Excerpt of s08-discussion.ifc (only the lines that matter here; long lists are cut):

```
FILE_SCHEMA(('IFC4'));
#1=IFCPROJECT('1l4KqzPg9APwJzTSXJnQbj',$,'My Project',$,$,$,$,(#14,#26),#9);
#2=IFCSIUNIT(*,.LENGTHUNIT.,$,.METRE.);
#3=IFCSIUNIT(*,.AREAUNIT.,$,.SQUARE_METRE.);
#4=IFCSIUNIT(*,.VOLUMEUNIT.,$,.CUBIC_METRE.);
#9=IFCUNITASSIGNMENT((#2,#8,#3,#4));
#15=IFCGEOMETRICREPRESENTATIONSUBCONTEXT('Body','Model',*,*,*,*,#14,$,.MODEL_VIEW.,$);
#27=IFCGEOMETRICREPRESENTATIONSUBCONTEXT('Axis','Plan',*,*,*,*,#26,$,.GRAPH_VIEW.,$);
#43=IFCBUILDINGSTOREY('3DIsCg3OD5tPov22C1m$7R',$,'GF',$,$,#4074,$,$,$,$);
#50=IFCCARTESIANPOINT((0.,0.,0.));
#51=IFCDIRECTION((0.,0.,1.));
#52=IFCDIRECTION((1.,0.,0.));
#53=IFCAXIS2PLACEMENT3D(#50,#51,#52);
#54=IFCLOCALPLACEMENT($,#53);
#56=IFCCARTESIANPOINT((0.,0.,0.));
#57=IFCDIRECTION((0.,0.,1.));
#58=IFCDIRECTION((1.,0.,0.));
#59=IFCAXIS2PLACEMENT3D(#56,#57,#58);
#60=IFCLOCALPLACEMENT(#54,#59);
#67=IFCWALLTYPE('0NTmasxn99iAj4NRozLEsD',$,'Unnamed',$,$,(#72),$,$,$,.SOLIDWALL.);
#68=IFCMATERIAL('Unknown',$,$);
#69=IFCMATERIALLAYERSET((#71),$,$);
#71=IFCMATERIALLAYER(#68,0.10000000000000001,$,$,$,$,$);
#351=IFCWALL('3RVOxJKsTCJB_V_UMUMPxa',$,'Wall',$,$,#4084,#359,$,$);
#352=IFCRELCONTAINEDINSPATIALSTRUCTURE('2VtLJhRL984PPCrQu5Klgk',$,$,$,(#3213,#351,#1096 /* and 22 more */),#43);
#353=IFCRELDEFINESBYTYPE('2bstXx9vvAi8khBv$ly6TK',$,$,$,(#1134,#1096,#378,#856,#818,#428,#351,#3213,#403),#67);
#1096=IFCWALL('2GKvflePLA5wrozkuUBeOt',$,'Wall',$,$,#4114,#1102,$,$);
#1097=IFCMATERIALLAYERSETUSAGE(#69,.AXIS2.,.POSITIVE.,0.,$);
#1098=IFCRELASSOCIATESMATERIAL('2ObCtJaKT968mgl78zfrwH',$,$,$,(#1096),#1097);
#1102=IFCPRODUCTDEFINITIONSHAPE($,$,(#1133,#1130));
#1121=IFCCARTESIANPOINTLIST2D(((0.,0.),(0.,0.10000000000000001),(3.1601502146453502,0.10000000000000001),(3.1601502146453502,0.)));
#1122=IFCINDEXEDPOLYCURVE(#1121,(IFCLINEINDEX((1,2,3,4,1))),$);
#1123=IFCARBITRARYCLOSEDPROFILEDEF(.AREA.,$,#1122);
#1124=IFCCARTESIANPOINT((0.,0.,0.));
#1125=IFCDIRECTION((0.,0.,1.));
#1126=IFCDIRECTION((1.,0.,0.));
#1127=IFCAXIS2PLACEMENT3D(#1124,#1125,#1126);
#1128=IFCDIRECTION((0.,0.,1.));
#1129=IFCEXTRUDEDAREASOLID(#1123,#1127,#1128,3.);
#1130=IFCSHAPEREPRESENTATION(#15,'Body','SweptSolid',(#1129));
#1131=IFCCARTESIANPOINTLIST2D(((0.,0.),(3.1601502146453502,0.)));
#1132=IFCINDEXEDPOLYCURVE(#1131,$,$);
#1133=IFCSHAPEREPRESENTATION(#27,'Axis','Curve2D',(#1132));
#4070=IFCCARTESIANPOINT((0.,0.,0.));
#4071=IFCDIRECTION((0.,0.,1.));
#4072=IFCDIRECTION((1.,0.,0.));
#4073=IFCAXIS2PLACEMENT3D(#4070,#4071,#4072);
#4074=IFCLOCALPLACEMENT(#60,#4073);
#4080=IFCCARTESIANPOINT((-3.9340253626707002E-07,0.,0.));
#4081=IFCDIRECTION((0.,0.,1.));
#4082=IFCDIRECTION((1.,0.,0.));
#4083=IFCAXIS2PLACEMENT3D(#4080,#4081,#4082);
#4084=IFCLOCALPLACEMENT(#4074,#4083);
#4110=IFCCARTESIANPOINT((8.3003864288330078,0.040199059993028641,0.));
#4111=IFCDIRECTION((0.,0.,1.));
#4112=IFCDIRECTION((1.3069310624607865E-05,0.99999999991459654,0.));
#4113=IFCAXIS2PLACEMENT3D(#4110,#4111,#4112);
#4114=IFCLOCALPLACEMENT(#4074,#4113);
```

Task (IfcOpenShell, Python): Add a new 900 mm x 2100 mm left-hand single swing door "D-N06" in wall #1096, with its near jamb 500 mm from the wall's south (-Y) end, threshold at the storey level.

```python
import numpy as np
import ifcopenshell
import ifcopenshell.api.feature
import ifcopenshell.api.geometry
import ifcopenshell.api.root
import ifcopenshell.api.spatial
import ifcopenshell.geom
import ifcopenshell.util.element
import ifcopenshell.util.placement
import ifcopenshell.util.representation
import ifcopenshell.util.shape
import ifcopenshell.util.unit

model = ifcopenshell.open("s08-discussion.ifc")
unit_scale = ifcopenshell.util.unit.calculate_unit_scale(model)
settings = ifcopenshell.geom.settings()


def volume(element):
    """Net volume in cubic metres, openings subtracted."""
    shape = ifcopenshell.geom.create_shape(settings, element)
    return ifcopenshell.util.shape.get_volume(shape.geometry)


wall = model.by_guid("2GKvflePLA5wrozkuUBeOt")
storey = ifcopenshell.util.element.get_container(wall, ifc_class="IfcBuildingStorey")
context = ifcopenshell.util.representation.get_context(model, "Model", "Body", "MODEL_VIEW")
before = volume(wall)

width, height, from_end, sill = 0.9, 2.1, 0.5, 0.0  # metres

# The wall runs along its own X axis, and the end named is its -X end.
wall_shape = ifcopenshell.geom.create_shape(settings, wall)
x, y, z = ifcopenshell.util.shape.get_vertices(wall_shape.geometry).T
start = x.min() + from_end
face, thickness = float(y.min()), float(y.max() - y.min())
wall_matrix = ifcopenshell.util.placement.get_local_placement(wall.ObjectPlacement)
level = ifcopenshell.util.placement.get_local_placement(storey.ObjectPlacement)[2, 3]


def in_wall(x, y):
    """Placement at x, y metres in the wall's axes, at sill height."""
    matrix = wall_matrix.copy()
    matrix[:, 3] = wall_matrix @ np.array([x / unit_scale, y / unit_scale, 0.0, 1.0])
    matrix[2, 3] = level + sill / unit_scale
    return matrix


# Opening: a box that overshoots both wall faces by 50 mm.
opening = ifcopenshell.api.root.create_entity(model, ifc_class="IfcOpeningElement", predefined_type="OPENING")
box = ifcopenshell.api.geometry.add_wall_representation(
    model, context=context, length=width, height=height, thickness=thickness + 0.1
)
ifcopenshell.api.geometry.assign_representation(model, product=opening, representation=box)
ifcopenshell.api.geometry.edit_object_placement(model, product=opening, matrix=in_wall(start, face - 0.05), is_si=False)
ifcopenshell.api.feature.add_feature(model, feature=opening, element=wall)

door = ifcopenshell.api.root.create_entity(model, ifc_class="IfcDoor", name="D-N06", predefined_type="DOOR")
door.OverallWidth, door.OverallHeight = width / unit_scale, height / unit_scale
door.OperationType = "SINGLE_SWING_LEFT"
body = ifcopenshell.api.geometry.add_door_representation(
    model,
    context=context,
    overall_width=door.OverallWidth,
    overall_height=door.OverallHeight,
    operation_type="SINGLE_SWING_LEFT",
    lining_properties={"LiningDepth": thickness / unit_scale, "ThresholdDepth": thickness / unit_scale},
)
ifcopenshell.api.geometry.assign_representation(model, product=door, representation=body)
ifcopenshell.api.spatial.assign_container(model, products=[door], relating_structure=storey)
ifcopenshell.api.feature.add_filling(model, opening=opening, element=door)

# The lining spans the wall, so the door starts at the wall face.
ifcopenshell.api.geometry.edit_object_placement(model, product=door, matrix=in_wall(start, face), is_si=False)

after = volume(wall)

print(f"wall volume {before:.3f} -> {after:.3f} m3")

model.write("s08-discussion_v2.ifc")
```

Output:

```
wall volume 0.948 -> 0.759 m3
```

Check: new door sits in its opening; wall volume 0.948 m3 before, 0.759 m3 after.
